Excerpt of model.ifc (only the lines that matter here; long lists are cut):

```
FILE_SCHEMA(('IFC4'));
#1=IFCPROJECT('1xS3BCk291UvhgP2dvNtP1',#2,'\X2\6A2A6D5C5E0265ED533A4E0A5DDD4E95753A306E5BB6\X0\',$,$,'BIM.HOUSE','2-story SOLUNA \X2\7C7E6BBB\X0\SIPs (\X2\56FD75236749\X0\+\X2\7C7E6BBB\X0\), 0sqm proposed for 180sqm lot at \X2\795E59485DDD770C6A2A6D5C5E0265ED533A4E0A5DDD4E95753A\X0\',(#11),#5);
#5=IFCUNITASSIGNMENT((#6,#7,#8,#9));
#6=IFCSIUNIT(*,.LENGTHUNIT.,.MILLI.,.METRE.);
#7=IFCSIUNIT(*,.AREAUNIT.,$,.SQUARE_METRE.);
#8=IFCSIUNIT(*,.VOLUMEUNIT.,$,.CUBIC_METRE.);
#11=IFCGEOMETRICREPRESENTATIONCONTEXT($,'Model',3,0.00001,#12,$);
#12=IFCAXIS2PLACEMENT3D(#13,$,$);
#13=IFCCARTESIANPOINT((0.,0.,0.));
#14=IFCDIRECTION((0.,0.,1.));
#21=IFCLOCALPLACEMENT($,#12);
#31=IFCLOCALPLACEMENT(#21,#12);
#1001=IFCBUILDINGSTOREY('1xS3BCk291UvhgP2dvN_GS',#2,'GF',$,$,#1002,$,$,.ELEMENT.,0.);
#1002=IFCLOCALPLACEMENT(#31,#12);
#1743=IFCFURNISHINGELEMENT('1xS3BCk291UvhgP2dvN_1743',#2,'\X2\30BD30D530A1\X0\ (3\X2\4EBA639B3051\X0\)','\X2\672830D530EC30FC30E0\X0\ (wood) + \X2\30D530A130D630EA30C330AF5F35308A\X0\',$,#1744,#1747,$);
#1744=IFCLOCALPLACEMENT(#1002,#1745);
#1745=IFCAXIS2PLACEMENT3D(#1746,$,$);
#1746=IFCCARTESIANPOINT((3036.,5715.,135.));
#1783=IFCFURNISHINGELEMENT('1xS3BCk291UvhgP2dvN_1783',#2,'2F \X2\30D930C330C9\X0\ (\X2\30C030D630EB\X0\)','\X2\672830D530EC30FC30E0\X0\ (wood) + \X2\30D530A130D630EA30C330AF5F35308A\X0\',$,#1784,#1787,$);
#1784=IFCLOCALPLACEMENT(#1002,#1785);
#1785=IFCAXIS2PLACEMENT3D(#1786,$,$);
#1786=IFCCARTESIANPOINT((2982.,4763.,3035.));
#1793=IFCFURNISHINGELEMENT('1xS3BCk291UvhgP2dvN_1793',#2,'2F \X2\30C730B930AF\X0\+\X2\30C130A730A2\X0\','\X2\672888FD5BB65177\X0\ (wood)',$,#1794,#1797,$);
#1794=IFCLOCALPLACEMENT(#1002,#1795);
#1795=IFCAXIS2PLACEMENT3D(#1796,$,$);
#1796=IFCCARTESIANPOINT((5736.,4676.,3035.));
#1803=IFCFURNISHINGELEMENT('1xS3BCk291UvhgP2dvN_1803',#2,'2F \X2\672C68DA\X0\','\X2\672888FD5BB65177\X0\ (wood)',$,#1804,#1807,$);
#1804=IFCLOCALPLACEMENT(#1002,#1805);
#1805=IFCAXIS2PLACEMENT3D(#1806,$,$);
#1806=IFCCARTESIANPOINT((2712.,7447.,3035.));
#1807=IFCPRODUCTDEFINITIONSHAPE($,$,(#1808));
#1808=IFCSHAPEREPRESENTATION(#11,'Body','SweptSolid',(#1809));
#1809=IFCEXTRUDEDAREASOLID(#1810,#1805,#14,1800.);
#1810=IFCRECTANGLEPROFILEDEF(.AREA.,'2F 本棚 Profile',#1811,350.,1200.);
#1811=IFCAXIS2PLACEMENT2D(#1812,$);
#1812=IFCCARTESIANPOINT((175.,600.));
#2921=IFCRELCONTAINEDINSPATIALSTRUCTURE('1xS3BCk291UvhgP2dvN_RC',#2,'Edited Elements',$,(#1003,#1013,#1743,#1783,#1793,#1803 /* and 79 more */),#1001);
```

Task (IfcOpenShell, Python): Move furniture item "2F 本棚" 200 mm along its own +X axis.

```python
import ifcopenshell
import ifcopenshell.api.geometry
import ifcopenshell.util.placement
import ifcopenshell.util.unit

model = ifcopenshell.open("model.ifc")
unit_scale = ifcopenshell.util.unit.calculate_unit_scale(model)

item = model.by_guid("1xS3BCk291UvhgP2dvN_1803")
matrix = ifcopenshell.util.placement.get_local_placement(item.ObjectPlacement)
matrix[:3, 3] += matrix[:3, 0] * 0.2 / unit_scale
ifcopenshell.api.geometry.edit_object_placement(model, product=item, matrix=matrix, is_si=False)

print(ifcopenshell.util.placement.get_local_placement(item.ObjectPlacement).round(3) + 0.0)

model.write("model_v2.ifc")
```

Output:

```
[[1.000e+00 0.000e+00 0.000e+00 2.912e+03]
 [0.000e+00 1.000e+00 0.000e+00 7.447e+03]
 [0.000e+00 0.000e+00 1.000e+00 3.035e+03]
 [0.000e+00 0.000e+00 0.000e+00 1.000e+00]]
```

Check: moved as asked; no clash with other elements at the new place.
